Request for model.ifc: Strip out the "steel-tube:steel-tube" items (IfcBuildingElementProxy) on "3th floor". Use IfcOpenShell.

First a look at what the model holds.

```python
import ifcopenshell
import ifcopenshell.util.element

model = ifcopenshell.open("model.ifc")
print(model.schema)
storey = next(s for s in model.by_type("IfcBuildingStorey") if s.Name == "3th floor")
proxies = [e for e in ifcopenshell.util.element.get_decomposition(storey) if e.is_a("IfcBuildingElementProxy")]
seen = {}
for e in proxies:
    element_type = ifcopenshell.util.element.get_type(e)
    name = element_type.Name if element_type not in (None, e) else None
    seen[name] = seen.get(name, 0) + 1
for name, count in sorted(seen.items(), key=str):
    print(count, "x", name)
```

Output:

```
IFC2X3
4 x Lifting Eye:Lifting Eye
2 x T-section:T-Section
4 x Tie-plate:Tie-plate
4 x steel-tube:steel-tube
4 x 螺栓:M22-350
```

```python
import ifcopenshell
import ifcopenshell.api.root
import ifcopenshell.util.element

model = ifcopenshell.open("model.ifc")

storey = next(s for s in model.by_type("IfcBuildingStorey") if s.Name == "3th floor")
proxies = [e for e in ifcopenshell.util.element.get_decomposition(storey) if e.is_a("IfcBuildingElementProxy")]
targets = [e for e in proxies if (t := ifcopenshell.util.element.get_type(e)) not in (None, e) and t.Name == "steel-tube:steel-tube"]

for e in targets:
    ifcopenshell.api.root.remove_product(model, product=e)
print(len(targets), "removed")

model.write("model_rev.ifc")
```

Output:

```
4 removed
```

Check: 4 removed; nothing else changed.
